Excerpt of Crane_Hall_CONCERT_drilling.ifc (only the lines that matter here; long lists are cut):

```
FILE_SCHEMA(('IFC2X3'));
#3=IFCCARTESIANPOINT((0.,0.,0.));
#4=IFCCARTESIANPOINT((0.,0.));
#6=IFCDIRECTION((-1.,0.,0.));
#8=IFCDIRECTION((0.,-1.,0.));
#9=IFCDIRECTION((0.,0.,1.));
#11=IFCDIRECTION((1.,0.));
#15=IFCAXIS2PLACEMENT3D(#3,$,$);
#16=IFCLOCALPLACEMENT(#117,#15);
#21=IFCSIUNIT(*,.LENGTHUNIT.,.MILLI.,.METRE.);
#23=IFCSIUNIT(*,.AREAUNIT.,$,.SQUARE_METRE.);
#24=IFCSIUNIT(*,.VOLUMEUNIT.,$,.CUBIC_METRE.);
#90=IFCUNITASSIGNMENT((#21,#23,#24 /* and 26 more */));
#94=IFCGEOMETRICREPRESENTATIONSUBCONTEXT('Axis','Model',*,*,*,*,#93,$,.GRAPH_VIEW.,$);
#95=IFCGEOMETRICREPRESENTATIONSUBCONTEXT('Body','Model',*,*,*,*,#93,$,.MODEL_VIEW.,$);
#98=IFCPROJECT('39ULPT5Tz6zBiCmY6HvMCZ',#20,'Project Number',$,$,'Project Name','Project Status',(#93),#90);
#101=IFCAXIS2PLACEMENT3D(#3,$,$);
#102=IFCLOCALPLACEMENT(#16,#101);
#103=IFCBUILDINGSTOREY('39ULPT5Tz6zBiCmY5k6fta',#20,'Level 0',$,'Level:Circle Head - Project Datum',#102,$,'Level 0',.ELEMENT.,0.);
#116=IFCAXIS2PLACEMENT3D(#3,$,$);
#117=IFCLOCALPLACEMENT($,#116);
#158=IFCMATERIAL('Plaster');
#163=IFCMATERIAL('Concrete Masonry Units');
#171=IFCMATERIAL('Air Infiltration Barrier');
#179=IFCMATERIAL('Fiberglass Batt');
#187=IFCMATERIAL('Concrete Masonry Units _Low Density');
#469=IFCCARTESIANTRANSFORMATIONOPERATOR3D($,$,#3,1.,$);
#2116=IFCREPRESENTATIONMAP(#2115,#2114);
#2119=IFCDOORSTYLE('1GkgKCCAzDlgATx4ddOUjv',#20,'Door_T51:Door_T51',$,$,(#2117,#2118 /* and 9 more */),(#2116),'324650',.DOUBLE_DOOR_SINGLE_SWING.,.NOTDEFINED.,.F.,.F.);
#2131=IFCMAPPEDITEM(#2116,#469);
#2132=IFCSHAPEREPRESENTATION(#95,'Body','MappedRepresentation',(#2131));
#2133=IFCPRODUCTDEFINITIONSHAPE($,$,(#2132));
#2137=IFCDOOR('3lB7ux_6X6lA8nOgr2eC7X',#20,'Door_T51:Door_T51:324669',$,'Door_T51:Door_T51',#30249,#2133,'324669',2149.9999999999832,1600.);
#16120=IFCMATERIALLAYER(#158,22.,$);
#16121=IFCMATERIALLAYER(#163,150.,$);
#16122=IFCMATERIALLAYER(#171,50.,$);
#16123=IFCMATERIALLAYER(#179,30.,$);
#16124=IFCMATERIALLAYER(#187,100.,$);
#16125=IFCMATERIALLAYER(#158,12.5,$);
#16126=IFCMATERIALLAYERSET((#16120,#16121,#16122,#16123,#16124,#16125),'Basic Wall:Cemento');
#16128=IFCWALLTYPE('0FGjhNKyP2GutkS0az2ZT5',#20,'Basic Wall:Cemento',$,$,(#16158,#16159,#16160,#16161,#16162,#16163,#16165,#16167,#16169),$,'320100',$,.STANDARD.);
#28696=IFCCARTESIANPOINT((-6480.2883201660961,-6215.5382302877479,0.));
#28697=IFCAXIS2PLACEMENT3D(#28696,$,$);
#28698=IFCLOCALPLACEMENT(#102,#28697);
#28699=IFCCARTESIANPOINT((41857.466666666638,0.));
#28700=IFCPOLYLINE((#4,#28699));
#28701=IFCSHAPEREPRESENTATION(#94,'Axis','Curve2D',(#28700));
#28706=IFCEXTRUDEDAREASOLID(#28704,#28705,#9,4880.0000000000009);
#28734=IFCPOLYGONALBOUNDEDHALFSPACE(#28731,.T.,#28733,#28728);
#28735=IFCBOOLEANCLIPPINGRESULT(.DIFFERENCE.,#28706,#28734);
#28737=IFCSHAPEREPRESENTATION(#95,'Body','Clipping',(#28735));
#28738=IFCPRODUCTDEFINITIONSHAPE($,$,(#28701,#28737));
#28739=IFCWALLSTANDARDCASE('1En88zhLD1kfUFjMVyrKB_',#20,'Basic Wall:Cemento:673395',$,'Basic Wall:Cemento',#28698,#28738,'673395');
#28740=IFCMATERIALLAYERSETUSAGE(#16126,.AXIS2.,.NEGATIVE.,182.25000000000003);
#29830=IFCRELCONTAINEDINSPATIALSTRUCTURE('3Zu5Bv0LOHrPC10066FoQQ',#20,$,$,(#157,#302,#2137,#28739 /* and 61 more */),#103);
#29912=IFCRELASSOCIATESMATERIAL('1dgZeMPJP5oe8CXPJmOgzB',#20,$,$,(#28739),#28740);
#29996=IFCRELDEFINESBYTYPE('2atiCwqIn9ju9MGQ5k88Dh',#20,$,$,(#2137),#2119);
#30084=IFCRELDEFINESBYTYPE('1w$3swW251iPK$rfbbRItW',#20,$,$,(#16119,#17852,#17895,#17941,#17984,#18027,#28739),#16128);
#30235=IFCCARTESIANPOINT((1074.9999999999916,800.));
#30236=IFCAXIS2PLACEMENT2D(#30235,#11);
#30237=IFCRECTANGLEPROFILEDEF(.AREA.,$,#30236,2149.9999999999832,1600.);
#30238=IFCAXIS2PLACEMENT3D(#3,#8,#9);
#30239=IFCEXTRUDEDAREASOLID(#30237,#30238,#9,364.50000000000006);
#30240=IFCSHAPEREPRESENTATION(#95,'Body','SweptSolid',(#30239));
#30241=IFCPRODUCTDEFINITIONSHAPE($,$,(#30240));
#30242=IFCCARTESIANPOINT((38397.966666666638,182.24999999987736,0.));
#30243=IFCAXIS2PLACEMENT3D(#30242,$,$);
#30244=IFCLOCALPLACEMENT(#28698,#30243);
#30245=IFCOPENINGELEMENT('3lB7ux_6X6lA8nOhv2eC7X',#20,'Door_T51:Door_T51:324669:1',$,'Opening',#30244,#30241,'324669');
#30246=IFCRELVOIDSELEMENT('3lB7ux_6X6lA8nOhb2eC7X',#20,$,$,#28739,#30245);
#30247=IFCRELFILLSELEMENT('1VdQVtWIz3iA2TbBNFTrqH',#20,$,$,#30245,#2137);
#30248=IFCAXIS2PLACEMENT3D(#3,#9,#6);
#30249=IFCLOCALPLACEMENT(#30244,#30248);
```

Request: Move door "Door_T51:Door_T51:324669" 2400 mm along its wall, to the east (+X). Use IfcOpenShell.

```python
import ifcopenshell
import ifcopenshell.api.geometry
import ifcopenshell.util.placement
import ifcopenshell.util.unit

model = ifcopenshell.open("Crane_Hall_CONCERT_drilling.ifc")
unit_scale = ifcopenshell.util.unit.calculate_unit_scale(model)

door = model.by_guid("3lB7ux_6X6lA8nOgr2eC7X")
opening = door.FillsVoids[0].RelatingOpeningElement
wall = opening.VoidsElements[0].RelatingBuildingElement

wall_matrix = ifcopenshell.util.placement.get_local_placement(wall.ObjectPlacement)
shift = wall_matrix[:3, 0] * 2.4 / unit_scale
before = ifcopenshell.util.placement.get_local_placement(door.ObjectPlacement)[:3, 3].copy()

# The door is placed relative to its opening, so it follows when the opening moves.
matrix = ifcopenshell.util.placement.get_local_placement(opening.ObjectPlacement)
matrix[:3, 3] += shift
ifcopenshell.api.geometry.edit_object_placement(
    model, product=opening, matrix=matrix, is_si=False, should_transform_children=True
)

after = ifcopenshell.util.placement.get_local_placement(door.ObjectPlacement)[:3, 3]
print("door moved by", (after - before).round(3) + 0.0)

model.write("Crane_Hall_CONCERT_drilling_rev.ifc")
```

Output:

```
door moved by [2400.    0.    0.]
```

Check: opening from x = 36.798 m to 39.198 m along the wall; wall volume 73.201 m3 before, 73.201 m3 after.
